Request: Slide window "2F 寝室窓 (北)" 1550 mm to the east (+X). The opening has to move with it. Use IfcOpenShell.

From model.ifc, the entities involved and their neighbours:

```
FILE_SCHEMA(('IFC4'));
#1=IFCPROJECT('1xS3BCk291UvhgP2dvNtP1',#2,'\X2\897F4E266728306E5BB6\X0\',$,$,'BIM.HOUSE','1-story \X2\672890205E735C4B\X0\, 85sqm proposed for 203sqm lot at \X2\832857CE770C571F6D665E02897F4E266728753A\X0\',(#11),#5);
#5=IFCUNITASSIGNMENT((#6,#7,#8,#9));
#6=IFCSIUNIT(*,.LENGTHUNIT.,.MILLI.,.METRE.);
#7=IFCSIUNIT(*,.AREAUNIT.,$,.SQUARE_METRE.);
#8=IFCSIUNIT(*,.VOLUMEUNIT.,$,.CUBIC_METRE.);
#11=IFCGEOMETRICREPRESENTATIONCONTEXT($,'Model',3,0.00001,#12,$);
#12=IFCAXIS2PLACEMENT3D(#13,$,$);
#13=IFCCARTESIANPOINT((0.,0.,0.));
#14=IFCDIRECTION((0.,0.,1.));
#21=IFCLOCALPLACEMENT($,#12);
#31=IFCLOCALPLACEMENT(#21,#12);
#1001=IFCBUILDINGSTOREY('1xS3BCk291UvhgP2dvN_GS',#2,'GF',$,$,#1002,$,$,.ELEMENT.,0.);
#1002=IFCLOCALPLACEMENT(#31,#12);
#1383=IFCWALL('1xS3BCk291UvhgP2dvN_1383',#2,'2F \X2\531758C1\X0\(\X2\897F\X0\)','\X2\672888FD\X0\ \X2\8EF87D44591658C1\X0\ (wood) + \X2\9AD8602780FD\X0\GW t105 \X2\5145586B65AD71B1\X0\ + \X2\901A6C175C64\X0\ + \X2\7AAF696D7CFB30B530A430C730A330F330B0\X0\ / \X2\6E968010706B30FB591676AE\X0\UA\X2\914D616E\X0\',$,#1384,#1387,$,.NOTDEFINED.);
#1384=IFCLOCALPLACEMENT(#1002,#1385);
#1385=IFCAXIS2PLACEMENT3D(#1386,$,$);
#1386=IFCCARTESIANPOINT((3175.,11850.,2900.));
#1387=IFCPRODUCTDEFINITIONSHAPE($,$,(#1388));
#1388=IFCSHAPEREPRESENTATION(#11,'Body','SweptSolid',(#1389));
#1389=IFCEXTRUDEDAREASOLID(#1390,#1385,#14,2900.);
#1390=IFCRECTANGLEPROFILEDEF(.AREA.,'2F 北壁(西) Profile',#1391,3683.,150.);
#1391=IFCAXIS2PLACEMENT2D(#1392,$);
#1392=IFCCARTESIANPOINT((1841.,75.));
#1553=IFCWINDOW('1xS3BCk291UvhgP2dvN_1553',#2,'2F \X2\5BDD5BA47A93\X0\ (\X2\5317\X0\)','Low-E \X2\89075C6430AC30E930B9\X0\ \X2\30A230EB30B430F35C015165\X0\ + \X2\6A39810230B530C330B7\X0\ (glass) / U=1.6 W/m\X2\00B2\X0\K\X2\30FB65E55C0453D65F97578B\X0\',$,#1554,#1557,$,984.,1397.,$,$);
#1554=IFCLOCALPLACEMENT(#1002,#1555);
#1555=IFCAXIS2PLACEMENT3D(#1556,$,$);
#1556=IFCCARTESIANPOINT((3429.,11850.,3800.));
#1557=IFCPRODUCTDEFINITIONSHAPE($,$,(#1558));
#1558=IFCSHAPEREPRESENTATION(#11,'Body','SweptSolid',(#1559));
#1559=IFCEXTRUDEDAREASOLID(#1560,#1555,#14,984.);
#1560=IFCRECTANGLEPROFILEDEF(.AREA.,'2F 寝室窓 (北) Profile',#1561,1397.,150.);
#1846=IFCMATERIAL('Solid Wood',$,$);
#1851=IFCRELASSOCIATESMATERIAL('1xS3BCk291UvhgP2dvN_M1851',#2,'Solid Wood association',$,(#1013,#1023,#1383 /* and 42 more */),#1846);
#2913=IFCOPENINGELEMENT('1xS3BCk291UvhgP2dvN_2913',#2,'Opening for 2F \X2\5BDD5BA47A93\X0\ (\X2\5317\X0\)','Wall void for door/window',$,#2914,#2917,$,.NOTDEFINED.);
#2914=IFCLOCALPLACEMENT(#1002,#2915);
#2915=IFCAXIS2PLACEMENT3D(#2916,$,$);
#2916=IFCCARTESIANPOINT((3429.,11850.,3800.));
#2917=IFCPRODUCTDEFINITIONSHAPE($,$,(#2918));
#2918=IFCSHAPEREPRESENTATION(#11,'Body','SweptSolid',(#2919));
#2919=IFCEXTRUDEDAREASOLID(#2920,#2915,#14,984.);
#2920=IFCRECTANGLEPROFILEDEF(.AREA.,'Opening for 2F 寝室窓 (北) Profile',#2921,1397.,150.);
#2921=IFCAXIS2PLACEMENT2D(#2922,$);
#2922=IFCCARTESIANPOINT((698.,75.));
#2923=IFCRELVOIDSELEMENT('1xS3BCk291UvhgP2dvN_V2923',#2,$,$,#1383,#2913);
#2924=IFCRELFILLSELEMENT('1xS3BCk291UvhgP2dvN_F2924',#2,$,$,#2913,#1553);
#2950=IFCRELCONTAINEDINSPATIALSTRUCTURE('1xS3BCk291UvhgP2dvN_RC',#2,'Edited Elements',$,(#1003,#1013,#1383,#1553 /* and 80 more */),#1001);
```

```python
import ifcopenshell
import ifcopenshell.api.geometry
import ifcopenshell.util.placement
import ifcopenshell.util.unit

model = ifcopenshell.open("model.ifc")
unit_scale = ifcopenshell.util.unit.calculate_unit_scale(model)

window = model.by_guid("1xS3BCk291UvhgP2dvN_1553")
opening = window.FillsVoids[0].RelatingOpeningElement
wall = opening.VoidsElements[0].RelatingBuildingElement

wall_matrix = ifcopenshell.util.placement.get_local_placement(wall.ObjectPlacement)
shift = wall_matrix[:3, 0] * 1.55 / unit_scale
before = ifcopenshell.util.placement.get_local_placement(window.ObjectPlacement)[:3, 3].copy()

# The window is not placed relative to its opening, so move both.
for product in (opening, window):
    matrix = ifcopenshell.util.placement.get_local_placement(product.ObjectPlacement)
    matrix[:3, 3] += shift
    ifcopenshell.api.geometry.edit_object_placement(model, product=product, matrix=matrix, is_si=False)

after = ifcopenshell.util.placement.get_local_placement(window.ObjectPlacement)[:3, 3]
print("window moved by", (after - before).round(3) + 0.0)

model.write("model_updated.ifc")
```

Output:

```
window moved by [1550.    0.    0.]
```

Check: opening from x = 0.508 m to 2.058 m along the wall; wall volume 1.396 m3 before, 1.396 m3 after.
